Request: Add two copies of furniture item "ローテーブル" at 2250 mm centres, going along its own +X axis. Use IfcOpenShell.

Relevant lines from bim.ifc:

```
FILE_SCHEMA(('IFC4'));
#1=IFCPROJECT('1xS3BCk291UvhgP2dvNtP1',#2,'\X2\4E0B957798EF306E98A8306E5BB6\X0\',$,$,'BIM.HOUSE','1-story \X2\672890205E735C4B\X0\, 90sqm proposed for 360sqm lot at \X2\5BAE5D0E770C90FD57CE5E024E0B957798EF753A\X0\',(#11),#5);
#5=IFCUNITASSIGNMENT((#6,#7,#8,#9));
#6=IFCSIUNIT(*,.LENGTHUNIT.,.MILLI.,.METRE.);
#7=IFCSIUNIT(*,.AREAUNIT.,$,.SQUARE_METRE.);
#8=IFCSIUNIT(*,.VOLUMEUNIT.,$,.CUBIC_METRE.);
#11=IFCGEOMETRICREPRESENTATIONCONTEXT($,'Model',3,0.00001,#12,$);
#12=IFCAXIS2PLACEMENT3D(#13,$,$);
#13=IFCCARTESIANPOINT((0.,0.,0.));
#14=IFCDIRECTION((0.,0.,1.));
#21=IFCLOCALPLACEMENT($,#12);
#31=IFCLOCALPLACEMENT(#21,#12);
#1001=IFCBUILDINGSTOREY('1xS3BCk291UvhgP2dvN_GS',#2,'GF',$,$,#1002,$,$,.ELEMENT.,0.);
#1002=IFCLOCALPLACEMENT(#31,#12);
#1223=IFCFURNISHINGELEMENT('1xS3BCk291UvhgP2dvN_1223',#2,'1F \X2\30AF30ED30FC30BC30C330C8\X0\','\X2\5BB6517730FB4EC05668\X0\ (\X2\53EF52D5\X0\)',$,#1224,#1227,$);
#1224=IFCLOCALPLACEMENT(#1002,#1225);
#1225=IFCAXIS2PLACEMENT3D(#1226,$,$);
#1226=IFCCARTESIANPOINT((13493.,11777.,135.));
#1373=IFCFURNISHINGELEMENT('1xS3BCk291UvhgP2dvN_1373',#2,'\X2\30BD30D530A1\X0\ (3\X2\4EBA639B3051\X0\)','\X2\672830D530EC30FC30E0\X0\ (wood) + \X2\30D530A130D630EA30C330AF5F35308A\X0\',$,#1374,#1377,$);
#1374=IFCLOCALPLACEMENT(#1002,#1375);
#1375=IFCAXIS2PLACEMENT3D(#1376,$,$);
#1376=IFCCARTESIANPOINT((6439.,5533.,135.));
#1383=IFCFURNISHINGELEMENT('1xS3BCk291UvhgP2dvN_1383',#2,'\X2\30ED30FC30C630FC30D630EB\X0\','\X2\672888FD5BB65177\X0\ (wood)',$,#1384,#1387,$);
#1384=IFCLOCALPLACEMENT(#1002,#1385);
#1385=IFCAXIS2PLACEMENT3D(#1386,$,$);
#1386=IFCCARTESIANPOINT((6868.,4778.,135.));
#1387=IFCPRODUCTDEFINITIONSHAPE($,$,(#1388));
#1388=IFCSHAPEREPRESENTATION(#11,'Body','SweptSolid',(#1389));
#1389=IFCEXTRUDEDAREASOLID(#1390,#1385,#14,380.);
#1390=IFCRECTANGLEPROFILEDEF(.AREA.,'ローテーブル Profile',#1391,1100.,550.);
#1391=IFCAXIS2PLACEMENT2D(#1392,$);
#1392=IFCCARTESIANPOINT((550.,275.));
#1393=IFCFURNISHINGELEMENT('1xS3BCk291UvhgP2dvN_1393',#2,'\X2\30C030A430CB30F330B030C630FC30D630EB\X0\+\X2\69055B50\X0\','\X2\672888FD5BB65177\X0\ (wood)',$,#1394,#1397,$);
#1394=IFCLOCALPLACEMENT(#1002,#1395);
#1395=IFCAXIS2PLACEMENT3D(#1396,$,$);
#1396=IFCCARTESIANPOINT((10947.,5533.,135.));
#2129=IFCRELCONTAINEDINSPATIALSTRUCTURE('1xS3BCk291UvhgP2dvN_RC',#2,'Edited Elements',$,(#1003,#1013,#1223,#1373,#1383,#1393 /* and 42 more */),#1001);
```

```python
import ifcopenshell
import ifcopenshell.api.geometry
import ifcopenshell.api.root
import ifcopenshell.util.element
import ifcopenshell.util.placement
import ifcopenshell.util.unit

model = ifcopenshell.open("bim.ifc")
unit_scale = ifcopenshell.util.unit.calculate_unit_scale(model)


def reuse_history(source, copy):
    """copy_class also copies each property set's owner history, people and application; keep the originals."""
    for rel in copy.IsDefinedBy:
        if rel.is_a("IfcRelDefinesByProperties") and (history := rel.RelatingPropertyDefinition.OwnerHistory):
            rel.RelatingPropertyDefinition.OwnerHistory = source.OwnerHistory
            ifcopenshell.util.element.remove_deep2(model, history)


source = model.by_guid("1xS3BCk291UvhgP2dvN_1383")
base = ifcopenshell.util.placement.get_local_placement(source.ObjectPlacement)
step = base[:3, 0] * 2.25 / unit_scale

for i in range(1, 3):
    copy = ifcopenshell.api.root.copy_class(model, product=source)
    copy.Representation = ifcopenshell.util.element.copy_deep(
        model, source.Representation, exclude=["IfcGeometricRepresentationContext", "IfcRepresentationMap"]
    )
    reuse_history(source, copy)
    matrix = base.copy()
    matrix[:3, 3] += i * step
    print("added at", matrix[:3, 3].round(3) + 0.0)
    ifcopenshell.api.geometry.edit_object_placement(model, product=copy, matrix=matrix, is_si=False)

model.write("bim_updated.ifc")
```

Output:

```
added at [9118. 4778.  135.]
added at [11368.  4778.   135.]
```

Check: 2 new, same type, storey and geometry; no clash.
